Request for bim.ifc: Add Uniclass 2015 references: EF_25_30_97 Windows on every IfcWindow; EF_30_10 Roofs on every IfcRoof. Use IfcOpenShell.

First a look at what the model holds.

```python
import ifcopenshell

model = ifcopenshell.open("bim.ifc")
print(model.schema)
print("classifications:", [c.Name for c in model.by_type("IfcClassification")])
for ifc_class in ("IfcDoor", "IfcRoof", "IfcStair", "IfcWall", "IfcWindow"):
    print(ifc_class, len(model.by_type(ifc_class)))
```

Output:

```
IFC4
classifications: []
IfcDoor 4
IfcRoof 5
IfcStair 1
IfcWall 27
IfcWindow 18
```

```python
import ifcopenshell
import ifcopenshell.api.classification

model = ifcopenshell.open("bim.ifc")

system = ifcopenshell.api.classification.add_classification(model, classification="Uniclass 2015")

codes = {
    "IfcWindow": ("EF_25_30_97", "Windows"),
    "IfcRoof": ("EF_30_10", "Roofs"),
}
for ifc_class, (code, name) in codes.items():
    products = model.by_type(ifc_class)
    ifcopenshell.api.classification.add_reference(
        model, products=products, classification=system, identification=code, name=name
    )
    print(code, len(products))

model.write("bim_rev.ifc")
```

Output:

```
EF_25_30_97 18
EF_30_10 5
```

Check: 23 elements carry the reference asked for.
